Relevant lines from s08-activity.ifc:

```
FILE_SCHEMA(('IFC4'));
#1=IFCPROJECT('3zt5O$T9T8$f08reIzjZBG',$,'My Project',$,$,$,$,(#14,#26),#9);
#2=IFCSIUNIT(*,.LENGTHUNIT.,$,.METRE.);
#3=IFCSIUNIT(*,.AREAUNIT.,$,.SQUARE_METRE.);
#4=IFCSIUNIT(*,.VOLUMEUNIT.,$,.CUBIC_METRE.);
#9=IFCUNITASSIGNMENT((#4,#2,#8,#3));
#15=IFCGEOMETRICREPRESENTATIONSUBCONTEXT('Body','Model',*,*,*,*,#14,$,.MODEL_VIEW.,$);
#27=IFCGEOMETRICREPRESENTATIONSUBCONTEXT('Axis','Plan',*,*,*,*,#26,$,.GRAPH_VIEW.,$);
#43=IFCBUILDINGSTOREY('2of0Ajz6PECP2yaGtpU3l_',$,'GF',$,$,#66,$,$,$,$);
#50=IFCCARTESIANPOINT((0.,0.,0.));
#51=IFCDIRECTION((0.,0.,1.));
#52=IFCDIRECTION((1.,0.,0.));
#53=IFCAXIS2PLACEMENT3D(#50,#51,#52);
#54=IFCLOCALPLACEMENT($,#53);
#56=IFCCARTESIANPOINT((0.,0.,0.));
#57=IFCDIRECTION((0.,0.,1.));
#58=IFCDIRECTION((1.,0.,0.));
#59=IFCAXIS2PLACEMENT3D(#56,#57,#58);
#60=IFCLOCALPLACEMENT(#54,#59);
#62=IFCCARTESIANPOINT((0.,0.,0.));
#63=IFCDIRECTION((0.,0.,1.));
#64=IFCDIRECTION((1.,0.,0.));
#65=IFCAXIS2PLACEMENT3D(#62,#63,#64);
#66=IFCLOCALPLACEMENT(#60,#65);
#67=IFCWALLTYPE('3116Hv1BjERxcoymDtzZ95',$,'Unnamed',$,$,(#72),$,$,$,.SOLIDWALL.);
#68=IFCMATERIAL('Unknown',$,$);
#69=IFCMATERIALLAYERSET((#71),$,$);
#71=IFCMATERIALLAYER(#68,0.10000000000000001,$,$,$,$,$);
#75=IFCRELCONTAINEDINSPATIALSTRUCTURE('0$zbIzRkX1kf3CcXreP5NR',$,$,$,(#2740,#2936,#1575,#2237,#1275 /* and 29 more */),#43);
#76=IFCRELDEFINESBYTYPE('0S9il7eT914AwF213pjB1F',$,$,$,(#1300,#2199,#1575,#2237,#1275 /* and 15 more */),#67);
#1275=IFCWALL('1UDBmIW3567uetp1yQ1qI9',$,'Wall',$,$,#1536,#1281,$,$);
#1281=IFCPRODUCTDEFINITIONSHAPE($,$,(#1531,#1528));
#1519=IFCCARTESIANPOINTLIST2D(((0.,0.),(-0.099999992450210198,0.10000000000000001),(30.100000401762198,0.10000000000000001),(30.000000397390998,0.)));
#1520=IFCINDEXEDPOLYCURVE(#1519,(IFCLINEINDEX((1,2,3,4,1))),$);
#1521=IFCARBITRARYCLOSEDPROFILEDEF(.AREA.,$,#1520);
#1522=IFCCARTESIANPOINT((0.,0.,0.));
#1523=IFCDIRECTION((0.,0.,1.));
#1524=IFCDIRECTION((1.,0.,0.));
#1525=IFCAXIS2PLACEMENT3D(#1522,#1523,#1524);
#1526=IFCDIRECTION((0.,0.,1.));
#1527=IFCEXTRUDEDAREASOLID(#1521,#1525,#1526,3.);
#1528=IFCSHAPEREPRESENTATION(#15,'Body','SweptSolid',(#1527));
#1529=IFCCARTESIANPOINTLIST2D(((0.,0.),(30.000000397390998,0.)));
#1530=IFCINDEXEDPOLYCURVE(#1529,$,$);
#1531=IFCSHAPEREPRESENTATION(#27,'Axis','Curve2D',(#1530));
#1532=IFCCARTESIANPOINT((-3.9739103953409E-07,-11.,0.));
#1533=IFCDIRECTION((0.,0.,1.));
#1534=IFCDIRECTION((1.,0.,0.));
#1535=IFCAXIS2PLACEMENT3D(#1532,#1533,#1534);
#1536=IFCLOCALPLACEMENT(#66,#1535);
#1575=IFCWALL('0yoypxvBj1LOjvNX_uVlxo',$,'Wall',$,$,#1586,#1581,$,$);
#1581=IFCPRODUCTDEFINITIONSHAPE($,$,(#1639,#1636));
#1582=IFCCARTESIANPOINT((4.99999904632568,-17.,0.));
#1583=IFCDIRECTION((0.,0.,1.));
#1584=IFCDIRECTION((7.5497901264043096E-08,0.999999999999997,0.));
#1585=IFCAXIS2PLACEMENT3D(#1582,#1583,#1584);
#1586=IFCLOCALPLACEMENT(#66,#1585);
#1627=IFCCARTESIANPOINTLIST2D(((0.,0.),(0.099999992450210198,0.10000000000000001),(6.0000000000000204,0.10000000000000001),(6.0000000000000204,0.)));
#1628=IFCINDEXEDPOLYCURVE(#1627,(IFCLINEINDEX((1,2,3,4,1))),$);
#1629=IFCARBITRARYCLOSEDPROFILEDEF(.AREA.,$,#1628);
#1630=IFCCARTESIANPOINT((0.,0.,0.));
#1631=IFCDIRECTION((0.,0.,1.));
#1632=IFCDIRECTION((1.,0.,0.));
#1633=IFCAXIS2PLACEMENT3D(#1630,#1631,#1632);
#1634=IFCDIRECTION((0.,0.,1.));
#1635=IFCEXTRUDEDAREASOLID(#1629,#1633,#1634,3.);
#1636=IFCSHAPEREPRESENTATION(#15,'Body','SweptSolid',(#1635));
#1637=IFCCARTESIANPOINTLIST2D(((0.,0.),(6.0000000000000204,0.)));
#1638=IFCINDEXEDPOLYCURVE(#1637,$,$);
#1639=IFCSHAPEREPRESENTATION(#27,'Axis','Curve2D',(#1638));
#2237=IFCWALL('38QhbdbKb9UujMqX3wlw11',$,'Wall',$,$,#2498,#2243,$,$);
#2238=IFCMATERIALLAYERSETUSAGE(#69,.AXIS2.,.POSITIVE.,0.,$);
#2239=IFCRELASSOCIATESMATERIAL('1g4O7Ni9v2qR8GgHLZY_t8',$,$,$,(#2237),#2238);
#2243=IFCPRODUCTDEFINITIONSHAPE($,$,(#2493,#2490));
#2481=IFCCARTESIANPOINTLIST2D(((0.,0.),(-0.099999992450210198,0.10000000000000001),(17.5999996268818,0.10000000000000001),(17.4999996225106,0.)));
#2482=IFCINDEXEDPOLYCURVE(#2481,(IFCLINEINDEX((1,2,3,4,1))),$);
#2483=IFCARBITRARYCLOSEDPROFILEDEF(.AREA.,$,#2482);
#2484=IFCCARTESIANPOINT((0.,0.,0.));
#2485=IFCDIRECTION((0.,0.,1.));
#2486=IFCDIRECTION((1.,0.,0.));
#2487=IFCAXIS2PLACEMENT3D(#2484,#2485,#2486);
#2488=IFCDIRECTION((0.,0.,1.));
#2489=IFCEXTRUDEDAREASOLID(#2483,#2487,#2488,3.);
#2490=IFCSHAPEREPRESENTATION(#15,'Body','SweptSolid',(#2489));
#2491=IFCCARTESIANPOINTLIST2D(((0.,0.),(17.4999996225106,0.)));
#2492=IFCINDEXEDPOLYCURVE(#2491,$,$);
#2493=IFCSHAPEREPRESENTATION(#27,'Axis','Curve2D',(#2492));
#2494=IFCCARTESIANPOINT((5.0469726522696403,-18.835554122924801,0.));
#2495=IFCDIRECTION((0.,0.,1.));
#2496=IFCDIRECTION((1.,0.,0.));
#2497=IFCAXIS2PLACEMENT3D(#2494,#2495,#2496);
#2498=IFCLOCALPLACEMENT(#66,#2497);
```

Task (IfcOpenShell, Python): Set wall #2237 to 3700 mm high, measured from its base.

```python
import ifcopenshell
import ifcopenshell.geom
import ifcopenshell.util.representation
import ifcopenshell.util.shape
import ifcopenshell.util.unit

model = ifcopenshell.open("s08-activity.ifc")
unit_scale = ifcopenshell.util.unit.calculate_unit_scale(model)
settings = ifcopenshell.geom.settings()


def volume(element):
    """Net volume in cubic metres, openings subtracted."""
    shape = ifcopenshell.geom.create_shape(settings, element)
    return ifcopenshell.util.shape.get_volume(shape.geometry)


wall = model.by_guid("38QhbdbKb9UujMqX3wlw11")
before = volume(wall)

body = ifcopenshell.util.representation.get_representation(wall, "Model", "Body")
solid = body.Items[0]
old_height = solid.Depth
solid.Depth = 3.7 / unit_scale
after = volume(wall)

print(f"height {old_height:g} -> {solid.Depth:g}, volume {before:.3f} -> {after:.3f} m3")

model.write("s08-activity-out.ifc")
```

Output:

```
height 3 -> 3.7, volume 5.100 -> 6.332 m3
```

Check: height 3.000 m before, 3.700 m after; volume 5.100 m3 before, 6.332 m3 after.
